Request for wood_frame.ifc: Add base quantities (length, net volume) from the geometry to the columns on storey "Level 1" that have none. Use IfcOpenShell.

First a look at what the model holds.

```python
import ifcopenshell
import ifcopenshell.util.element
import ifcopenshell.util.unit

model = ifcopenshell.open("wood_frame.ifc")
print(model.schema)
for unit_type in ("LENGTHUNIT", "AREAUNIT", "VOLUMEUNIT"):
    print(unit_type, ifcopenshell.util.unit.calculate_unit_scale(model, unit_type))
storey = next(s for s in model.by_type("IfcBuildingStorey") if s.Name == "Level 1")
columns = [e for e in ifcopenshell.util.element.get_decomposition(storey) if e.is_a("IfcColumn")]
for e in sorted(columns, key=lambda e: e.id()):
    print(e.id(), e.is_a(), e.Name, list(ifcopenshell.util.element.get_psets(e, qtos_only=True)), sep=" | ")
```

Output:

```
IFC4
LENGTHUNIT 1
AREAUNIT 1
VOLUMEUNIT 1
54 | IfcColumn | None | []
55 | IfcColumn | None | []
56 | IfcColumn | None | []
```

```python
import ifcopenshell
import ifcopenshell.api.pset
import ifcopenshell.geom
import ifcopenshell.util.element
import ifcopenshell.util.shape
import ifcopenshell.util.unit

model = ifcopenshell.open("wood_frame.ifc")
unit_scale = ifcopenshell.util.unit.calculate_unit_scale(model)
volume_scale = ifcopenshell.util.unit.calculate_unit_scale(model, "VOLUMEUNIT")
settings = ifcopenshell.geom.settings()

storey = next(s for s in model.by_type("IfcBuildingStorey") if s.Name == "Level 1")
columns = [e for e in ifcopenshell.util.element.get_decomposition(storey) if e.is_a("IfcColumn")]

for e in sorted(columns, key=lambda e: e.id()):
    if ifcopenshell.util.element.get_psets(e, qtos_only=True, should_inherit=False):
        continue
    # Geometry comes back in metres, in the element's own axes.
    shape = ifcopenshell.geom.create_shape(settings, e)
    values = {
        "Length": ifcopenshell.util.shape.get_z(shape.geometry) / unit_scale,
        "NetVolume": ifcopenshell.util.shape.get_volume(shape.geometry) / volume_scale,
    }
    qto = ifcopenshell.api.pset.add_qto(model, product=e, name="Qto_ColumnBaseQuantities")
    ifcopenshell.api.pset.edit_qto(model, qto=qto, properties=values)
    print(e.id(), {k: round(v, 3) for k, v in values.items()})

model.write("wood_frame_updated.ifc")
```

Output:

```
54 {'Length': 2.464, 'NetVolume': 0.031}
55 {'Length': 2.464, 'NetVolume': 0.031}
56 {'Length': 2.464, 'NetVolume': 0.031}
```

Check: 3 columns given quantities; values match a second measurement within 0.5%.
